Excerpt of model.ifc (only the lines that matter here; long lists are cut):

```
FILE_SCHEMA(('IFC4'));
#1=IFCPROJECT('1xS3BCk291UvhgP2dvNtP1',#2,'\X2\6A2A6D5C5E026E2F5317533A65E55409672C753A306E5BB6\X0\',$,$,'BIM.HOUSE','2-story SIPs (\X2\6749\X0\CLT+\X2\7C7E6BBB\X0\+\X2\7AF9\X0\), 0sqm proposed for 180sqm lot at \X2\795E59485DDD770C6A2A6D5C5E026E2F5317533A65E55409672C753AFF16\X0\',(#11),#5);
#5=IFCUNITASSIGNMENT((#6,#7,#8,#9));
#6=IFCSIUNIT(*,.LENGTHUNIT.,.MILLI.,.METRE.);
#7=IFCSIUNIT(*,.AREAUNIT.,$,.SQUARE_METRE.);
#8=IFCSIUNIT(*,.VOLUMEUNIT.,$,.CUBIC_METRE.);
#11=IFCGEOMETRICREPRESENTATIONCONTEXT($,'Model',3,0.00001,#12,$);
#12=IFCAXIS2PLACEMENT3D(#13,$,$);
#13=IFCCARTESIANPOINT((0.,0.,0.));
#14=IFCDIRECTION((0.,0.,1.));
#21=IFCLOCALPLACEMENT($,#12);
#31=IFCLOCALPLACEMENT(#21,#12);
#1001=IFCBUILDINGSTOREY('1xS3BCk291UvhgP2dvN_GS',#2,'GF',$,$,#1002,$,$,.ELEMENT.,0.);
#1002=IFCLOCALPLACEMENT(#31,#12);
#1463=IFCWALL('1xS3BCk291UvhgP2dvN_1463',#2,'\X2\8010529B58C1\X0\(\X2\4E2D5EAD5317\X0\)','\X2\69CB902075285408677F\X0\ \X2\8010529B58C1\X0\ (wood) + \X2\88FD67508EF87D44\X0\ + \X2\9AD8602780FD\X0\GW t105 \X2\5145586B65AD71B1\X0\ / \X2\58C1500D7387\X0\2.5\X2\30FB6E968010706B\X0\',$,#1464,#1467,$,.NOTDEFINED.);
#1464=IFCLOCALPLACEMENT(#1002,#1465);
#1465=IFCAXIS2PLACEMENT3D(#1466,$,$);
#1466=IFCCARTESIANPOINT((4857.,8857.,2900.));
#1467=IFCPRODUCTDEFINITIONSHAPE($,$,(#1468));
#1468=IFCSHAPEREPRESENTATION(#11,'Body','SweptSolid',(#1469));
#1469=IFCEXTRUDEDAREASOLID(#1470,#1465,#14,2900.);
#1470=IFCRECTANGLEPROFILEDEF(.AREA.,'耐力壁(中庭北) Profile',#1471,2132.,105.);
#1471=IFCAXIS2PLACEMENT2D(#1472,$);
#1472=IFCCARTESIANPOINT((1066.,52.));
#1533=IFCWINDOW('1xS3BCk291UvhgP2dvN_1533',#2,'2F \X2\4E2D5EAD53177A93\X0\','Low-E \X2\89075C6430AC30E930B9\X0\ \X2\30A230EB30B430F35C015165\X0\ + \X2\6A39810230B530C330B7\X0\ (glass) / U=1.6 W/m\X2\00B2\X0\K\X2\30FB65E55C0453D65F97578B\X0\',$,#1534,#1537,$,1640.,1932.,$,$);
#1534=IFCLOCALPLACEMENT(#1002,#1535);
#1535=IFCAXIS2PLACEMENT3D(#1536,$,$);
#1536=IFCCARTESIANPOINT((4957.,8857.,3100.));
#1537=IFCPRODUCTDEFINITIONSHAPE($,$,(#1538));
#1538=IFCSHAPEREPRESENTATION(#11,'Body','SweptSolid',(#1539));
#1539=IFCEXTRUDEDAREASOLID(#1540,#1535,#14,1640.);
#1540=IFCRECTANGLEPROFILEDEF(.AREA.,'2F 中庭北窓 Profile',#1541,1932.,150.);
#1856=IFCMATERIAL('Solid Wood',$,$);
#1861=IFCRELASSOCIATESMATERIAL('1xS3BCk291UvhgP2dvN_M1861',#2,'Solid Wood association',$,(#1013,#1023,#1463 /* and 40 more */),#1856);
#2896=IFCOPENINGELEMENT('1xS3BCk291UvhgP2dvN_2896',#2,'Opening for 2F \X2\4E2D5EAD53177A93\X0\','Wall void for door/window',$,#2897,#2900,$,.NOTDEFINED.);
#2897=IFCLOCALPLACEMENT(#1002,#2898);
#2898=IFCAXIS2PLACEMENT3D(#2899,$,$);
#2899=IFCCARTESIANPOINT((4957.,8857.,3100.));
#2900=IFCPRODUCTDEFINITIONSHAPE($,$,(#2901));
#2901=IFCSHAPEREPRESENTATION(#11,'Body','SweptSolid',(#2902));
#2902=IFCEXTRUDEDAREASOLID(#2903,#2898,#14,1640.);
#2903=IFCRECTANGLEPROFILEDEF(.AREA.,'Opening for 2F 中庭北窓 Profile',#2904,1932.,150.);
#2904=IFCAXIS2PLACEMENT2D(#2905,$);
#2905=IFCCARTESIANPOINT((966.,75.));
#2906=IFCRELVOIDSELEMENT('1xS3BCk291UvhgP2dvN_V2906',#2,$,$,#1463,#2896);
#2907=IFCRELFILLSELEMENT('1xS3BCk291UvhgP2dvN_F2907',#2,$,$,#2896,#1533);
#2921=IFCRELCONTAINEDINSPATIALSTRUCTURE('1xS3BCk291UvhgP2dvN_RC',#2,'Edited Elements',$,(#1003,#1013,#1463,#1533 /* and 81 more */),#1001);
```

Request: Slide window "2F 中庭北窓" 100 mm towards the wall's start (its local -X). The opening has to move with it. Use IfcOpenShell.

```python
import ifcopenshell
import ifcopenshell.api.geometry
import ifcopenshell.util.placement
import ifcopenshell.util.unit

model = ifcopenshell.open("model.ifc")
unit_scale = ifcopenshell.util.unit.calculate_unit_scale(model)

window = model.by_guid("1xS3BCk291UvhgP2dvN_1533")
opening = window.FillsVoids[0].RelatingOpeningElement
wall = opening.VoidsElements[0].RelatingBuildingElement

wall_matrix = ifcopenshell.util.placement.get_local_placement(wall.ObjectPlacement)
shift = wall_matrix[:3, 0] * -0.1 / unit_scale
before = ifcopenshell.util.placement.get_local_placement(window.ObjectPlacement)[:3, 3].copy()

# The window is not placed relative to its opening, so move both.
for product in (opening, window):
    matrix = ifcopenshell.util.placement.get_local_placement(product.ObjectPlacement)
    matrix[:3, 3] += shift
    ifcopenshell.api.geometry.edit_object_placement(model, product=product, matrix=matrix, is_si=False)

after = ifcopenshell.util.placement.get_local_placement(window.ObjectPlacement)[:3, 3]
print("window moved by", (after - before).round(3) + 0.0)

model.write("model_updated.ifc")
```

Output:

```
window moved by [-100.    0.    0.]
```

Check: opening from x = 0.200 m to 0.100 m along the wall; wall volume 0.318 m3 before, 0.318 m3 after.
